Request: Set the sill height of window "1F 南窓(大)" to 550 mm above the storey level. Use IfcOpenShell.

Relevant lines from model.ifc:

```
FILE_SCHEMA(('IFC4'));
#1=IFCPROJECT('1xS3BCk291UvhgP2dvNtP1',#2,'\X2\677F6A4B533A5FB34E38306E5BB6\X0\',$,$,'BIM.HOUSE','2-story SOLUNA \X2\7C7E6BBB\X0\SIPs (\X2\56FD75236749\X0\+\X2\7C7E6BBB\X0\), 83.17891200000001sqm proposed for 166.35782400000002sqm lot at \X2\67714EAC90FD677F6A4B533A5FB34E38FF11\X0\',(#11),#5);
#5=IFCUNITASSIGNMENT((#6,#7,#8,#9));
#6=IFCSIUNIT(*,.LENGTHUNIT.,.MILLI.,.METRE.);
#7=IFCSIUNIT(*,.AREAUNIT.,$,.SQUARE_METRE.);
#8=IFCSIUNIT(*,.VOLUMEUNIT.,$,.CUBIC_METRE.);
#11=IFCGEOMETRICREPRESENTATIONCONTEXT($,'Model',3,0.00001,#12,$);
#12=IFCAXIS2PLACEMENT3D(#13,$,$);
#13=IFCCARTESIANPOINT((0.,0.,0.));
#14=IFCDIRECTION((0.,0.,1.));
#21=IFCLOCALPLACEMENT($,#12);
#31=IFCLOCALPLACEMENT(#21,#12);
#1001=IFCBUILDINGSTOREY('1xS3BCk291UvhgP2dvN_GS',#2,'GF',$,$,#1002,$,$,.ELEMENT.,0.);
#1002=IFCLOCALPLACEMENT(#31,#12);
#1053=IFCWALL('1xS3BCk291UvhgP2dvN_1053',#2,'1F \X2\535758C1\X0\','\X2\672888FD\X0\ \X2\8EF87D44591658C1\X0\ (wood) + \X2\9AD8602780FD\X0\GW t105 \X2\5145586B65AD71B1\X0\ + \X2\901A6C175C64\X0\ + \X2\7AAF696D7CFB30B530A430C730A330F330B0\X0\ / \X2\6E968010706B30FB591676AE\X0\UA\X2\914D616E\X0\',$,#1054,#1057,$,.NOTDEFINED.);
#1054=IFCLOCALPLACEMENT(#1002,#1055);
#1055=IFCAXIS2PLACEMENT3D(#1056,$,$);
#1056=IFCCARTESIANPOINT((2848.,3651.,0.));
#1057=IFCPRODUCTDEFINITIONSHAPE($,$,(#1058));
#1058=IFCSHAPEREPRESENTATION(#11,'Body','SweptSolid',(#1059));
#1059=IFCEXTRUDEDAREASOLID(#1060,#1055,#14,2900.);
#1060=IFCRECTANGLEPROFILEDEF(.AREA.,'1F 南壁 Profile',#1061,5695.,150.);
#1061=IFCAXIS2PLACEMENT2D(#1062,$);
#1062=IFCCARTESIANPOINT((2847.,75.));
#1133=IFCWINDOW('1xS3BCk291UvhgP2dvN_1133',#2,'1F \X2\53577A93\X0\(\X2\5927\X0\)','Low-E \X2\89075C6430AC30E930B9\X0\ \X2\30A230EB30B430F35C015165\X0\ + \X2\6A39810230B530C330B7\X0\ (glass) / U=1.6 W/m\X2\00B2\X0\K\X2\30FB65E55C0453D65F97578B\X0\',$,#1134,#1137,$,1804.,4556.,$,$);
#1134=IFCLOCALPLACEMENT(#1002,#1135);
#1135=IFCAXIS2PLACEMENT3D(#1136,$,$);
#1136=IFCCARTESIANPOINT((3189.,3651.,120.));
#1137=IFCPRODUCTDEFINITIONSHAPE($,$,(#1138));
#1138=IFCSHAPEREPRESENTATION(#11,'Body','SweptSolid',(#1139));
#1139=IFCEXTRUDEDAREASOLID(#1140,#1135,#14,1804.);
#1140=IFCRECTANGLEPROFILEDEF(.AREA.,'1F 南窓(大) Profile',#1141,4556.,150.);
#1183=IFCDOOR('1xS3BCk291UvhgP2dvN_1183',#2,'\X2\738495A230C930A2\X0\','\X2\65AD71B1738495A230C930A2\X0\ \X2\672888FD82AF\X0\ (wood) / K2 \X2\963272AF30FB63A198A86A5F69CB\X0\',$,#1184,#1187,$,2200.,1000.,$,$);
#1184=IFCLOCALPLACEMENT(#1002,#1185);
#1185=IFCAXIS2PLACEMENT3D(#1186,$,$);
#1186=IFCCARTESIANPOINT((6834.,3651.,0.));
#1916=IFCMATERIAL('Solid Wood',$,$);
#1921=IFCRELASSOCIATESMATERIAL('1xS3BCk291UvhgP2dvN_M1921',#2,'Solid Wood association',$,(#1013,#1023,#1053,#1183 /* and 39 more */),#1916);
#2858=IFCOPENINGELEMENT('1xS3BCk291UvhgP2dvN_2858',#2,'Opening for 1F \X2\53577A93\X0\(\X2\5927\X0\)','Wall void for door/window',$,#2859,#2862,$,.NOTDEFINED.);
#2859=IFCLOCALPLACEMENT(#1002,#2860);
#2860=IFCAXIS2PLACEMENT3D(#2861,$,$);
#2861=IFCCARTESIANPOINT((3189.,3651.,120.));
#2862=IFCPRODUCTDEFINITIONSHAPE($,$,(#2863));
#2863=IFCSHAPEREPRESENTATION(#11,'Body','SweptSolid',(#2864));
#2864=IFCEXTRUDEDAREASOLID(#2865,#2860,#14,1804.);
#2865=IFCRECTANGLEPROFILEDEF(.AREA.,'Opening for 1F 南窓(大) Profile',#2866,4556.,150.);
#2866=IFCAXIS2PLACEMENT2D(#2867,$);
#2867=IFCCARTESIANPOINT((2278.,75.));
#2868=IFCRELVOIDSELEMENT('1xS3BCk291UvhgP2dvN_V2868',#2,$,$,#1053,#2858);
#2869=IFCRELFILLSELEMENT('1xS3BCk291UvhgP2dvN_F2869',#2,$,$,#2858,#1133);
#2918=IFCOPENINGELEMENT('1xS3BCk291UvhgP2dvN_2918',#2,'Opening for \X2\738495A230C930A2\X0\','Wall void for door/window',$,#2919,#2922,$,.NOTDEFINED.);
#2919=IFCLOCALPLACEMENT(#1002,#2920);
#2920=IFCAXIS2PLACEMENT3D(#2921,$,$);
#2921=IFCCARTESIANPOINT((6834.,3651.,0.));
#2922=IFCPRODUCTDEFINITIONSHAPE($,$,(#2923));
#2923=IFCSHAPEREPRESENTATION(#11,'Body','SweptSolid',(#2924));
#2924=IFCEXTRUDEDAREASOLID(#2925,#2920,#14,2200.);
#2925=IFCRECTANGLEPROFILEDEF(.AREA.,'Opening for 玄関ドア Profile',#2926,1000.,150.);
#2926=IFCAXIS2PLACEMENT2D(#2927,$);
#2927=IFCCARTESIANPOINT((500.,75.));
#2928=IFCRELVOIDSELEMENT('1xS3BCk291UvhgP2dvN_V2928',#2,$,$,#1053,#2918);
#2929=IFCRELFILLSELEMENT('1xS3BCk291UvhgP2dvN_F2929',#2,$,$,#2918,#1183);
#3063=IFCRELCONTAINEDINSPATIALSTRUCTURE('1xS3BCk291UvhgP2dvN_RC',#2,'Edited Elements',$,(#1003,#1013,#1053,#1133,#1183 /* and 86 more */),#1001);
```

```python
import numpy as np
import ifcopenshell
import ifcopenshell.api.geometry
import ifcopenshell.geom
import ifcopenshell.util.element
import ifcopenshell.util.placement
import ifcopenshell.util.shape
import ifcopenshell.util.unit

model = ifcopenshell.open("model.ifc")
unit_scale = ifcopenshell.util.unit.calculate_unit_scale(model)

window = model.by_guid("1xS3BCk291UvhgP2dvN_1133")
opening = window.FillsVoids[0].RelatingOpeningElement
storey = ifcopenshell.util.element.get_container(window, ifc_class="IfcBuildingStorey")
level = ifcopenshell.util.placement.get_local_placement(storey.ObjectPlacement)[2, 3]

# The opening's origin need not be at the sill, so measure its lowest point.
shape = ifcopenshell.geom.create_shape(ifcopenshell.geom.settings(), opening)
bottom = ifcopenshell.util.shape.get_shape_bottom_elevation(shape, shape.geometry) / unit_scale
dz = level + 0.55 / unit_scale - bottom

shift = np.array([0.0, 0.0, dz])
# The window is not placed relative to its opening, so move both.
for product in (opening, window):
    matrix = ifcopenshell.util.placement.get_local_placement(product.ObjectPlacement)
    matrix[:3, 3] += shift
    ifcopenshell.api.geometry.edit_object_placement(model, product=product, matrix=matrix, is_si=False)

print(f"moved by {dz * unit_scale:+.3f} m")

model.write("model_edited.ifc")
```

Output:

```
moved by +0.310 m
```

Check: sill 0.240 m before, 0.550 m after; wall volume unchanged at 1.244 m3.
